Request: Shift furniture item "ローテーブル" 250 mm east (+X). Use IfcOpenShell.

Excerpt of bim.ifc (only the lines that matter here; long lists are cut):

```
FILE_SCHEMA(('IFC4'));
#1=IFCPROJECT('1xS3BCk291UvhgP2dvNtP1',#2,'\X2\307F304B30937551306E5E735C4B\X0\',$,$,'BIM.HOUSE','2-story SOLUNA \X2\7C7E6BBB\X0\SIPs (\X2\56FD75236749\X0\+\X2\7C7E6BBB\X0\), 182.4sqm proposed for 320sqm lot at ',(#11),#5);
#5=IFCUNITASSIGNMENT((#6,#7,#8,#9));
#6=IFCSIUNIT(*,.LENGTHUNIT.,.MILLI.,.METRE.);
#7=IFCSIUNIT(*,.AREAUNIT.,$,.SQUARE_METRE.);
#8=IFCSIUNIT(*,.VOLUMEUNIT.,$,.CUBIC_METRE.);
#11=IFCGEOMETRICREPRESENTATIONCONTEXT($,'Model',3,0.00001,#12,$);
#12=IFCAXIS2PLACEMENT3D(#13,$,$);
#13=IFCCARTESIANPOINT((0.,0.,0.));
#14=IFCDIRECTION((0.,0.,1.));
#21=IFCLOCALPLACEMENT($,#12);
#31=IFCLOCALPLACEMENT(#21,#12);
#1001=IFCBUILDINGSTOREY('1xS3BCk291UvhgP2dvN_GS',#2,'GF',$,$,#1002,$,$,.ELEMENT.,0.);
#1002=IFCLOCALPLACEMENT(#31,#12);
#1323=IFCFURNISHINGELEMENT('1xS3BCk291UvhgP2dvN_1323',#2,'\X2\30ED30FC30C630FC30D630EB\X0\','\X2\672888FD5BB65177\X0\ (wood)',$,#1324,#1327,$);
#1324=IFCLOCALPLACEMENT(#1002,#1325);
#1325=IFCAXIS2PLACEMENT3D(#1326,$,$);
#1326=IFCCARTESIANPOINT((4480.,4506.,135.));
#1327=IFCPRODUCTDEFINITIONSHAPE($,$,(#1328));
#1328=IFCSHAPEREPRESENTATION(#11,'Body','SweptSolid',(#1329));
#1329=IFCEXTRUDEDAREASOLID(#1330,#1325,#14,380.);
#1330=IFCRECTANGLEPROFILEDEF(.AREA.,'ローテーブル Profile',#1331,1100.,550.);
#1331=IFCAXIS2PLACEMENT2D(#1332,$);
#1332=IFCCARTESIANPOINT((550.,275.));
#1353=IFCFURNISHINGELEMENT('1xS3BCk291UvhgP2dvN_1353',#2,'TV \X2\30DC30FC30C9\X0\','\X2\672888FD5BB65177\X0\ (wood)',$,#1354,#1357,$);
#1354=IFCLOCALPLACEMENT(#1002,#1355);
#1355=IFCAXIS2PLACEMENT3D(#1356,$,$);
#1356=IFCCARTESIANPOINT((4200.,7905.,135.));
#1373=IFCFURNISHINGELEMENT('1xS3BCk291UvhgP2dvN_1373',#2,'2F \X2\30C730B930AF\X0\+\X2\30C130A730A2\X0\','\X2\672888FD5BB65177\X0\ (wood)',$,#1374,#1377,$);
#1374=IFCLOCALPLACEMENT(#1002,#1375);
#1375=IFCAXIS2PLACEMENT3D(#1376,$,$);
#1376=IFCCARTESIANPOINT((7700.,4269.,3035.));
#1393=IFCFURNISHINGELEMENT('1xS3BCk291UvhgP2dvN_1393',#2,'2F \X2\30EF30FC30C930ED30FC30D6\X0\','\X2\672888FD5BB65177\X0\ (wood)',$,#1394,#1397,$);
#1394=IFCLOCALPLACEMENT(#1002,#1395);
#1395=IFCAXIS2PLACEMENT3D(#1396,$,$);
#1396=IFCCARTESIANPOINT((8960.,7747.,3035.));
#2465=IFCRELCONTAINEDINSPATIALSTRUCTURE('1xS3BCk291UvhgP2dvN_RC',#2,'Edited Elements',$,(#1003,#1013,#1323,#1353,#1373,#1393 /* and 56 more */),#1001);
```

```python
import ifcopenshell
import ifcopenshell.api.geometry
import ifcopenshell.util.placement

model = ifcopenshell.open("bim.ifc")

item = model.by_guid("1xS3BCk291UvhgP2dvN_1323")
matrix = ifcopenshell.util.placement.get_local_placement(item.ObjectPlacement)
matrix[0, 3] += 250.0
ifcopenshell.api.geometry.edit_object_placement(model, product=item, matrix=matrix, is_si=False)

print(ifcopenshell.util.placement.get_local_placement(item.ObjectPlacement).round(3) + 0.0)

model.write("bim_rev.ifc")
```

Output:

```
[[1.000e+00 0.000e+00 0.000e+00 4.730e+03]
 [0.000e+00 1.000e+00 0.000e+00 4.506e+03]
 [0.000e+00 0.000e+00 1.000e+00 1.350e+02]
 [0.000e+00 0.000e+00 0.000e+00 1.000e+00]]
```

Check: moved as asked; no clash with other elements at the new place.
